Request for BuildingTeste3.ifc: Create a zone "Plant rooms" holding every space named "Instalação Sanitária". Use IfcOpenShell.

First a look at what the model holds.

```python
import ifcopenshell

model = ifcopenshell.open("BuildingTeste3.ifc")
print(model.schema)
seen = {}
for space in model.by_type("IfcSpace"):
    seen[space.LongName] = seen.get(space.LongName, 0) + 1
for name, count in sorted(seen.items(), key=str):
    print(count, "x", name)
print("zones:", [z.Name for z in model.by_type("IfcZone")][:20])
```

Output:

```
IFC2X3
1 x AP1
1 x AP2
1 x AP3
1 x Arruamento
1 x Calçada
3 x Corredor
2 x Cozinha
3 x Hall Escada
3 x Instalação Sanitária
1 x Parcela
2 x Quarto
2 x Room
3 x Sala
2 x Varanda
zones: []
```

```python
import ifcopenshell
import ifcopenshell.api.group
import ifcopenshell.api.root

model = ifcopenshell.open("BuildingTeste3.ifc")

names = {"Instalação Sanitária"}
spaces = [s for s in model.by_type("IfcSpace") if s.LongName in names]

zone = ifcopenshell.api.root.create_entity(model, ifc_class="IfcZone", name="Plant rooms")
ifcopenshell.api.group.assign_group(model, products=spaces, group=zone)
print(len(spaces), "spaces in", zone.Name)

model.write("BuildingTeste3-out.ifc")
```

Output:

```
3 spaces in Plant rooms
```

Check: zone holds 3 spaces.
